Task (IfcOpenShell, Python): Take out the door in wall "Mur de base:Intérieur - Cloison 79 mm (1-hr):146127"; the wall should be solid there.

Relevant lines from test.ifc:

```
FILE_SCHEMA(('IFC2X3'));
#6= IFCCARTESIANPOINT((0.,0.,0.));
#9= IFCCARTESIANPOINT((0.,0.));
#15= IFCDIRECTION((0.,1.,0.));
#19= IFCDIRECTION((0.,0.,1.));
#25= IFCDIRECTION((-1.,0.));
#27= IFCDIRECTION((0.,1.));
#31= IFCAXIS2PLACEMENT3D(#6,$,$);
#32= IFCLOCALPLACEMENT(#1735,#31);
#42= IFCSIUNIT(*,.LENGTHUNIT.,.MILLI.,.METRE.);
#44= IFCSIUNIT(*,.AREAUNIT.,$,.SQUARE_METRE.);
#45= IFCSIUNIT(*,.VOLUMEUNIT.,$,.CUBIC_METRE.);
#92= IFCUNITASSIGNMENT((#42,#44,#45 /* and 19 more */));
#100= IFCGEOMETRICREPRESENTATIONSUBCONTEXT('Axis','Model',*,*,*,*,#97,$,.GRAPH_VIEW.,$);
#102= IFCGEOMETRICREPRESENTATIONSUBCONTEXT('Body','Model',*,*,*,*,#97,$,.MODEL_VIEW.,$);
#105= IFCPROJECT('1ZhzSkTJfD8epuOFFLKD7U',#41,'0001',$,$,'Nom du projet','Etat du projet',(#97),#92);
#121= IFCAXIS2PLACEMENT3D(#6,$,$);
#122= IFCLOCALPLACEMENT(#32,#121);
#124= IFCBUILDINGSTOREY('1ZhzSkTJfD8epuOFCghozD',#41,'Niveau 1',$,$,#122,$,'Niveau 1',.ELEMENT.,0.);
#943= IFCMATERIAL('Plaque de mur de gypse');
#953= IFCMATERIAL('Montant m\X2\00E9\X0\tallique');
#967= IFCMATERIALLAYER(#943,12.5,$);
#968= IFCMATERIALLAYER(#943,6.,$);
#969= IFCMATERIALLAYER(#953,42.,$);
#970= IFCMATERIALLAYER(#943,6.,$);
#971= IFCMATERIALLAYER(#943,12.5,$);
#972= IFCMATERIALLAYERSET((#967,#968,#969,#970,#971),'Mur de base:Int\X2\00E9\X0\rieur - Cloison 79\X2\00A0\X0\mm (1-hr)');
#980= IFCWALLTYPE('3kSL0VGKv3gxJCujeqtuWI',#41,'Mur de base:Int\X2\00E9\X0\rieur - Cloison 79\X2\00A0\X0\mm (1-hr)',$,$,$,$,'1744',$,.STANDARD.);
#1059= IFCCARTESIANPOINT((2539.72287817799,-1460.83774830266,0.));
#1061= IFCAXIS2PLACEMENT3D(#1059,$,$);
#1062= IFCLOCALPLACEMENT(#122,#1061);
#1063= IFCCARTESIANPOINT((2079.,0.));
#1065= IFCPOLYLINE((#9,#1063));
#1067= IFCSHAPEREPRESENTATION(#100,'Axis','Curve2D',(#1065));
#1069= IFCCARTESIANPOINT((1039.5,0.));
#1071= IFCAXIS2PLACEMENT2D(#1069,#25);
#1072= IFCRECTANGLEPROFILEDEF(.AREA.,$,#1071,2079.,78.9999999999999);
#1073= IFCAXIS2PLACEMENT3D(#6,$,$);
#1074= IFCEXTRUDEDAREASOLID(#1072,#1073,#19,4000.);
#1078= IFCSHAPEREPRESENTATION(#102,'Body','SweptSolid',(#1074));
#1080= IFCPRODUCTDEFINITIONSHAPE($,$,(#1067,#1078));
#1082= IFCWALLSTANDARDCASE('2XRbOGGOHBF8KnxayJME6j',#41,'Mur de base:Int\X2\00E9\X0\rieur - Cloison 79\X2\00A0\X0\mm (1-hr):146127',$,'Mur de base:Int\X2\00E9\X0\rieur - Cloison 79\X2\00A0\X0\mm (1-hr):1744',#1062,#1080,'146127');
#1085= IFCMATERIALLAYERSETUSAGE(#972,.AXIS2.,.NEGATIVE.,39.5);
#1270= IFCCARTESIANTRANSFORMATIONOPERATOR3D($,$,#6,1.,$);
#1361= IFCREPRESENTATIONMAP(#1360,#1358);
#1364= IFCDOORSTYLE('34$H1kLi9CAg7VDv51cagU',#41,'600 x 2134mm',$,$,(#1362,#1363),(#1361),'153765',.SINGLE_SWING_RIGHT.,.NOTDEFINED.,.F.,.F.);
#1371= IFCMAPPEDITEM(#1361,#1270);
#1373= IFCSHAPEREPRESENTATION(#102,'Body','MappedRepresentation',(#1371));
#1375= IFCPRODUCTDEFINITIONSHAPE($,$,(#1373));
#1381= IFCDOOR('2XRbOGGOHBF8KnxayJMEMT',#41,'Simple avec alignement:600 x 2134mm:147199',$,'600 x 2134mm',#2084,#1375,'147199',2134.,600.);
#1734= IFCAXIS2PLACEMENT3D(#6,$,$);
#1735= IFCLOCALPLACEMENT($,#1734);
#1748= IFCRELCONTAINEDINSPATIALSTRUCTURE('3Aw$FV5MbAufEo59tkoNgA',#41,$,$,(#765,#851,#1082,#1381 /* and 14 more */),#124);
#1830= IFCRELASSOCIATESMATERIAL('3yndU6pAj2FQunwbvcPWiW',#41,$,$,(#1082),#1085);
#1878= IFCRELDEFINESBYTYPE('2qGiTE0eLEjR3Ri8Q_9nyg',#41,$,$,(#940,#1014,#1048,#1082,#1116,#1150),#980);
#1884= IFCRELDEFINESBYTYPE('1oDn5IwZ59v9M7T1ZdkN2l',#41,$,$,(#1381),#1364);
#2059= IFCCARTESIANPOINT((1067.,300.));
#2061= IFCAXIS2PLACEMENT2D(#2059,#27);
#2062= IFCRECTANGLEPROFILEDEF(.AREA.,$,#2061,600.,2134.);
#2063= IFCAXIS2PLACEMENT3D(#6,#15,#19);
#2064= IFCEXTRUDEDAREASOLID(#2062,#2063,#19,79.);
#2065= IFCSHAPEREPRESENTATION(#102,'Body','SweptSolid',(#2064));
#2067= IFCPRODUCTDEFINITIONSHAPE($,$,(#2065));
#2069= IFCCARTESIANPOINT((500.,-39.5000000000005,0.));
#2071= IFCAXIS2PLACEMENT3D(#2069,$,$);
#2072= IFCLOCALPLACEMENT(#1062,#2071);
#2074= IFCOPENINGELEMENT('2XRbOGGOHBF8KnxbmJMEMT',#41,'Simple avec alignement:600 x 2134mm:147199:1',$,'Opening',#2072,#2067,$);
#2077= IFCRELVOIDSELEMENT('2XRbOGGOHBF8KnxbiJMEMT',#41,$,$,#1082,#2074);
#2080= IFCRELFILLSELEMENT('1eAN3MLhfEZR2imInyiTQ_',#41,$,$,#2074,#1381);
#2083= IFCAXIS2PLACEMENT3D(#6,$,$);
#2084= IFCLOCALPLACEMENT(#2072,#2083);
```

```python
import ifcopenshell
import ifcopenshell.api.feature
import ifcopenshell.api.root
import ifcopenshell.geom
import ifcopenshell.util.shape

model = ifcopenshell.open("test.ifc")
settings = ifcopenshell.geom.settings()


def volume(element):
    """Net volume in cubic metres, openings subtracted."""
    shape = ifcopenshell.geom.create_shape(settings, element)
    return ifcopenshell.util.shape.get_volume(shape.geometry)


door = model.by_guid("2XRbOGGOHBF8KnxayJMEMT")
opening = door.FillsVoids[0].RelatingOpeningElement
wall = opening.VoidsElements[0].RelatingBuildingElement
before = volume(wall)

ifcopenshell.api.root.remove_product(model, product=door)
ifcopenshell.api.feature.remove_feature(model, feature=opening)

after = volume(wall)

print(f"wall volume {before:.3f} -> {after:.3f} m3")

model.write("test-out.ifc")
```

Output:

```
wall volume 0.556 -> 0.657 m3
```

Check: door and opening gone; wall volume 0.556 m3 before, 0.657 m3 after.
